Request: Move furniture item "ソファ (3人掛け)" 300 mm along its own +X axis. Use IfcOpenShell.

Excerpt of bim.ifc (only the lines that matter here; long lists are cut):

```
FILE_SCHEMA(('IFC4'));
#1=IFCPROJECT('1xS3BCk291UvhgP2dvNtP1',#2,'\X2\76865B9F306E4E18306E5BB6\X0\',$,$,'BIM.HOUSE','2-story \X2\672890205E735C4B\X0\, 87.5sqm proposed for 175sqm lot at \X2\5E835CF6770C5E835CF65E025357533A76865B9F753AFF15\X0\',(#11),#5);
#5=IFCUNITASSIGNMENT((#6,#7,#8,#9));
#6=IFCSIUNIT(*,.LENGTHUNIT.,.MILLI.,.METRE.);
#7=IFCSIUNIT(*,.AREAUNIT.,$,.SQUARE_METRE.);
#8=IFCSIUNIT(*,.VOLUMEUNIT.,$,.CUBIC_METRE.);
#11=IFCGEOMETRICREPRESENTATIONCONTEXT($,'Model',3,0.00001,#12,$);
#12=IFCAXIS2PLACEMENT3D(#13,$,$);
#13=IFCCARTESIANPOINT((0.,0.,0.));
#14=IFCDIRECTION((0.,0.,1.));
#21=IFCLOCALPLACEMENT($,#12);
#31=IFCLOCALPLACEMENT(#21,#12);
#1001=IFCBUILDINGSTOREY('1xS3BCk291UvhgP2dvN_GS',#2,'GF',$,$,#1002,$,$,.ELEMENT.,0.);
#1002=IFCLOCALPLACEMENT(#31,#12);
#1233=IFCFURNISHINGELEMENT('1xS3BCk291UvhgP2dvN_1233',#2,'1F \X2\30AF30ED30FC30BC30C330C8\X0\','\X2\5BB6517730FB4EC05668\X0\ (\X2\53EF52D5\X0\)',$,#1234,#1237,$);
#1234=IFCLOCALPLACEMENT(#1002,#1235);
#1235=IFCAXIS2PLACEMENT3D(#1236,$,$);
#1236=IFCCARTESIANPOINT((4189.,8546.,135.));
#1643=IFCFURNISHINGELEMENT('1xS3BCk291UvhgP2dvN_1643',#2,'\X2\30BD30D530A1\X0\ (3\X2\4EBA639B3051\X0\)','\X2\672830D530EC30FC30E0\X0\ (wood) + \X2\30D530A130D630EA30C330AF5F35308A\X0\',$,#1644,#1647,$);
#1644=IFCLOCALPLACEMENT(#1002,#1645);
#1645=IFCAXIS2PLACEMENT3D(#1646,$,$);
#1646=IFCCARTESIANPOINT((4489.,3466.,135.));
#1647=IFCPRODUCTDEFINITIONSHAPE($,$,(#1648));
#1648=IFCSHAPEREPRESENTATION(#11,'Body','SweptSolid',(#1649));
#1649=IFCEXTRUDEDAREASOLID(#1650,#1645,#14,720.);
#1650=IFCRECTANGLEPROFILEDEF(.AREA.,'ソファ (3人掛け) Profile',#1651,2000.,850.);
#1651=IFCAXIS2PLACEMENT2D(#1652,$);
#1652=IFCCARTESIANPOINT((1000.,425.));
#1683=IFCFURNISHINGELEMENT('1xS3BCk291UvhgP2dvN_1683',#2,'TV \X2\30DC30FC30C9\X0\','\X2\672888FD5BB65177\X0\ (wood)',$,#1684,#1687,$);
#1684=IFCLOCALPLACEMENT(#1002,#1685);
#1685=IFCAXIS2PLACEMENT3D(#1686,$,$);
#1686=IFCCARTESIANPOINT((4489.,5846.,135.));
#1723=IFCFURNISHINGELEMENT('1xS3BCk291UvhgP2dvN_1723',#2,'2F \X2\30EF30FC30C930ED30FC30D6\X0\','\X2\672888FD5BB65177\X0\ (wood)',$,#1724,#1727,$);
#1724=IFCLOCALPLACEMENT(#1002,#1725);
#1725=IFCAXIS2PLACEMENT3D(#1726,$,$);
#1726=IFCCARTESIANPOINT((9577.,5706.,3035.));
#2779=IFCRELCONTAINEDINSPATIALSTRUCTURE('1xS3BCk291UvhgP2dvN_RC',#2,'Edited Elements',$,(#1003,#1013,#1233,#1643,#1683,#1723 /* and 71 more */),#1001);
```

```python
import ifcopenshell
import ifcopenshell.api.geometry
import ifcopenshell.util.placement
import ifcopenshell.util.unit

model = ifcopenshell.open("bim.ifc")
unit_scale = ifcopenshell.util.unit.calculate_unit_scale(model)

item = model.by_guid("1xS3BCk291UvhgP2dvN_1643")
matrix = ifcopenshell.util.placement.get_local_placement(item.ObjectPlacement)
matrix[:3, 3] += matrix[:3, 0] * 0.3 / unit_scale
ifcopenshell.api.geometry.edit_object_placement(model, product=item, matrix=matrix, is_si=False)

print(ifcopenshell.util.placement.get_local_placement(item.ObjectPlacement).round(3) + 0.0)

model.write("bim_updated.ifc")
```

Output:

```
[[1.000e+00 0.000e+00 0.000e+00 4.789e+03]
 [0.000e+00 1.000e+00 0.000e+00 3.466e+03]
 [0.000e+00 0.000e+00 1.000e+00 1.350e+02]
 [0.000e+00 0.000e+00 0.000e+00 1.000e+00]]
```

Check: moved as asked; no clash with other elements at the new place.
